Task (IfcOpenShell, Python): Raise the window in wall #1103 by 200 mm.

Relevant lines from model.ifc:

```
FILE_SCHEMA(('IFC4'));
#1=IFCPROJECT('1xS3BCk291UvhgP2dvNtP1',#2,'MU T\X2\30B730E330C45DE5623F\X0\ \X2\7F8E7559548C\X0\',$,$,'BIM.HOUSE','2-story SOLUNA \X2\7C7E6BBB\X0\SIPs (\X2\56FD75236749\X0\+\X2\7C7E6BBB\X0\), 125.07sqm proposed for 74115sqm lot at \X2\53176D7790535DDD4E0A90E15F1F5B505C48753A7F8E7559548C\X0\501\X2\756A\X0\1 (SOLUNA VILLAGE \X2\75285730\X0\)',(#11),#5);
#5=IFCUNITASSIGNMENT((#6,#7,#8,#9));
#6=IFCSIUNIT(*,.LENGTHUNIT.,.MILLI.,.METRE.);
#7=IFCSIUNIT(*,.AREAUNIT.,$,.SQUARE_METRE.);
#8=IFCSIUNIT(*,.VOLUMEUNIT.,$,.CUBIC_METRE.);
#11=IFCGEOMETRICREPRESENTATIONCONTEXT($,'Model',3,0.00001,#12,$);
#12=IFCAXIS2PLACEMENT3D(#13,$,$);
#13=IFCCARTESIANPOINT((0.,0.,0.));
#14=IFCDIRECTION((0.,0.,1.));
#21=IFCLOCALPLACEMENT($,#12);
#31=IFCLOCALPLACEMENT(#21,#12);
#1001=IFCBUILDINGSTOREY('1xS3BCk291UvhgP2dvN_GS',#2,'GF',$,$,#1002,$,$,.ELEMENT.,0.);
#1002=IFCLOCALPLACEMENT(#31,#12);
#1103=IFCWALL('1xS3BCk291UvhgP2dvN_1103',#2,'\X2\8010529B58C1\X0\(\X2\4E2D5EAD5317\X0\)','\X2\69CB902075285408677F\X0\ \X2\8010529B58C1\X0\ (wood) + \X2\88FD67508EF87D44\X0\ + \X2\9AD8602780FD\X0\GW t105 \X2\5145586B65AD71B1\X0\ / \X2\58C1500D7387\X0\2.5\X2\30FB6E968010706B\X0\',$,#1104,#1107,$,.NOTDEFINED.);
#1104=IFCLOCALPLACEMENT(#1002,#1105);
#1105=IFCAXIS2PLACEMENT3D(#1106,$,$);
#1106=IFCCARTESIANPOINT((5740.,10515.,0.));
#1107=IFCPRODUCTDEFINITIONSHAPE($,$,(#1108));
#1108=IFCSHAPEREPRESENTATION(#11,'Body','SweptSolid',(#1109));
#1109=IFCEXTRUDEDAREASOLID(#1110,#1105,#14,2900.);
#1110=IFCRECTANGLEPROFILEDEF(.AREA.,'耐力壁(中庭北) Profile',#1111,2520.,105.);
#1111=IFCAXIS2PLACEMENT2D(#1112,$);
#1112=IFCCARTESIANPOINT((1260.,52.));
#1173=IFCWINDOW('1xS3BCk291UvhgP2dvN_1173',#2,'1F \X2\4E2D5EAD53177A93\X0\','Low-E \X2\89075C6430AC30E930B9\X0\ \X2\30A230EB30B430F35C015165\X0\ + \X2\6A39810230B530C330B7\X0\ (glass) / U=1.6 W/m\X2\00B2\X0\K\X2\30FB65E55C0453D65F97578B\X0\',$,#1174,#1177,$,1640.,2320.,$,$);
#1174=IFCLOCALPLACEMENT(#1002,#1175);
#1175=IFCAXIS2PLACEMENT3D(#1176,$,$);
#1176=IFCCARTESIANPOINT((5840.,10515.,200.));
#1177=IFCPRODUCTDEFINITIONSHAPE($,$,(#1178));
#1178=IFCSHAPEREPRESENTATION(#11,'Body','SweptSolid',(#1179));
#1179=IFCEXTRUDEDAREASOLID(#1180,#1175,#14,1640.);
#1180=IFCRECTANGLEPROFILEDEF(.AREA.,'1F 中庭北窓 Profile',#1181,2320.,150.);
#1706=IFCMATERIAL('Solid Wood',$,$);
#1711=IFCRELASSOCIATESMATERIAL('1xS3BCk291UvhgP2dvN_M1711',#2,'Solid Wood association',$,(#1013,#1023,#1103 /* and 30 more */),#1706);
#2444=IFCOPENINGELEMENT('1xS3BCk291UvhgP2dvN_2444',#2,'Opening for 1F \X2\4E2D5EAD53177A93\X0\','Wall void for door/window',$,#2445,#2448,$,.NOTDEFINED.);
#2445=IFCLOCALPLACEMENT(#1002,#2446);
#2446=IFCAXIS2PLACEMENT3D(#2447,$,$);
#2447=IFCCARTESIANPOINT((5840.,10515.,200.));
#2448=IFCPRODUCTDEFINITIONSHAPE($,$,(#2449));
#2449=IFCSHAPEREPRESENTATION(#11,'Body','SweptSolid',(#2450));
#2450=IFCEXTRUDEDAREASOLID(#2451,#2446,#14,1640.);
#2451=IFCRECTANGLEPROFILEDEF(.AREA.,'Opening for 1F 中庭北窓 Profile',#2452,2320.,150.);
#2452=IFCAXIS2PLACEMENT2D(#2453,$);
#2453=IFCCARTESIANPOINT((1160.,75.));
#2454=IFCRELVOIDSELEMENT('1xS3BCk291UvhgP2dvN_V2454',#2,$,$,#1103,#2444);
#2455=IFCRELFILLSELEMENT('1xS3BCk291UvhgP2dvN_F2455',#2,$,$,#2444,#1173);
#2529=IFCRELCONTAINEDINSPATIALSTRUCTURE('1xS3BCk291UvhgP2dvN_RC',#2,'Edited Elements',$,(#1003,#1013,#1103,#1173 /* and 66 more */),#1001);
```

```python
import numpy as np
import ifcopenshell
import ifcopenshell.api.geometry
import ifcopenshell.util.placement
import ifcopenshell.util.unit

model = ifcopenshell.open("model.ifc")
unit_scale = ifcopenshell.util.unit.calculate_unit_scale(model)

window = model.by_id(1173)
opening = window.FillsVoids[0].RelatingOpeningElement
dz = 0.2 / unit_scale

shift = np.array([0.0, 0.0, dz])
# The window is not placed relative to its opening, so move both.
for product in (opening, window):
    matrix = ifcopenshell.util.placement.get_local_placement(product.ObjectPlacement)
    matrix[:3, 3] += shift
    ifcopenshell.api.geometry.edit_object_placement(model, product=product, matrix=matrix, is_si=False)

print(f"moved by {dz * unit_scale:+.3f} m")

model.write("model_v2.ifc")
```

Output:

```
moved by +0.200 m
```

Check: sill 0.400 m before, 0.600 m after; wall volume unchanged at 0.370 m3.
